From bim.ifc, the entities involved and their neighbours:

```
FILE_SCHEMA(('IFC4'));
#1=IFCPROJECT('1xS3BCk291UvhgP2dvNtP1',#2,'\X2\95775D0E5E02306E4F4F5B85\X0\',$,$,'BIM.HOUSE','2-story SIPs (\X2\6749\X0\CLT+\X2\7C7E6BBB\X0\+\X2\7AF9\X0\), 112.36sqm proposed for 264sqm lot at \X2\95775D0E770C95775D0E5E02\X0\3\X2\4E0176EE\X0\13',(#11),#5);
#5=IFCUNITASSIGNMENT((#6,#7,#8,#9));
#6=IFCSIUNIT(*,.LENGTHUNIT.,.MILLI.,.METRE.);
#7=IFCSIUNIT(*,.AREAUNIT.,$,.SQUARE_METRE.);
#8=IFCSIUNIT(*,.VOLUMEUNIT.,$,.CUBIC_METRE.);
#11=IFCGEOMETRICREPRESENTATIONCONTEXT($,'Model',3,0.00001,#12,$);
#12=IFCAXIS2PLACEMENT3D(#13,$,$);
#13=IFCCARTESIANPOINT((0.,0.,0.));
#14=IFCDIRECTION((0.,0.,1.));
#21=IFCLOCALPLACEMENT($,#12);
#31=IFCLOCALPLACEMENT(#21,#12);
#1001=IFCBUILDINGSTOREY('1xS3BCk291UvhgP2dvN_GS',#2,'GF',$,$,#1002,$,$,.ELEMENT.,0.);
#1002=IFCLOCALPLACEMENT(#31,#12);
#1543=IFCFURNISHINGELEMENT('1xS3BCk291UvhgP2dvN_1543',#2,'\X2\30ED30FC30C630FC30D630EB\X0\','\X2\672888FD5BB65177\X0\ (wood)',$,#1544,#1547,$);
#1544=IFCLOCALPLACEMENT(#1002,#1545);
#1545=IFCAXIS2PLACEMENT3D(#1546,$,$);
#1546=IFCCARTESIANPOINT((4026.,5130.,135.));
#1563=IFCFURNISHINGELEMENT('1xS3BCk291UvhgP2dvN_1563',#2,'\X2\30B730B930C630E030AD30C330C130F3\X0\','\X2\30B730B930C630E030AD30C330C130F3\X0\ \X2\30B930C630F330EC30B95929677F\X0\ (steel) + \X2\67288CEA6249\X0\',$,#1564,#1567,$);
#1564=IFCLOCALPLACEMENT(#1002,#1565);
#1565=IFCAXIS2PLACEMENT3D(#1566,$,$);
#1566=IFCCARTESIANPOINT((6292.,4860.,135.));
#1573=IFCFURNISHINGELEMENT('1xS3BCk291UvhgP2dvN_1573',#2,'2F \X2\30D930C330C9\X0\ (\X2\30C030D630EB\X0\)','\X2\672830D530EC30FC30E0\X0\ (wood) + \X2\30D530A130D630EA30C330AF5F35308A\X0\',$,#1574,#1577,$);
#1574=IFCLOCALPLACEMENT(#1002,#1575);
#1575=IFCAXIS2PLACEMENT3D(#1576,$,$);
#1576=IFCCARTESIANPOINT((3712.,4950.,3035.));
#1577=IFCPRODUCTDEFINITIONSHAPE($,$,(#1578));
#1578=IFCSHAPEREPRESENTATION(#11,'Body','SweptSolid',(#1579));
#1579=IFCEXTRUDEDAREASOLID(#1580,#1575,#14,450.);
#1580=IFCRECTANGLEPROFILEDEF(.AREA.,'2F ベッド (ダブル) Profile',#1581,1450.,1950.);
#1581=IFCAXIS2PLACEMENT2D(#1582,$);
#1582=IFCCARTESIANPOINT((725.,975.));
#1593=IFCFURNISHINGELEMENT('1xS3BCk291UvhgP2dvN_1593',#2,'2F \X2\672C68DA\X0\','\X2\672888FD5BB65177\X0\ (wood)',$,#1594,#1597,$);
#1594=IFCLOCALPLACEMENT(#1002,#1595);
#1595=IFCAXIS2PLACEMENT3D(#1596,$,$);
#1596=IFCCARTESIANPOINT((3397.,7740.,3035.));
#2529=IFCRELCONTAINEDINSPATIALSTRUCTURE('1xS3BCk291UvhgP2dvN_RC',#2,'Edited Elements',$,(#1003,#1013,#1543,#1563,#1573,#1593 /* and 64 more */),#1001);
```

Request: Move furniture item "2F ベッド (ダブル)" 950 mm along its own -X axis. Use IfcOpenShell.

```python
import ifcopenshell
import ifcopenshell.api.geometry
import ifcopenshell.util.placement
import ifcopenshell.util.unit

model = ifcopenshell.open("bim.ifc")
unit_scale = ifcopenshell.util.unit.calculate_unit_scale(model)

item = model.by_id(1573)
matrix = ifcopenshell.util.placement.get_local_placement(item.ObjectPlacement)
matrix[:3, 3] -= matrix[:3, 0] * 0.95 / unit_scale
ifcopenshell.api.geometry.edit_object_placement(model, product=item, matrix=matrix, is_si=False)

print(ifcopenshell.util.placement.get_local_placement(item.ObjectPlacement).round(3) + 0.0)

model.write("bim_edited.ifc")
```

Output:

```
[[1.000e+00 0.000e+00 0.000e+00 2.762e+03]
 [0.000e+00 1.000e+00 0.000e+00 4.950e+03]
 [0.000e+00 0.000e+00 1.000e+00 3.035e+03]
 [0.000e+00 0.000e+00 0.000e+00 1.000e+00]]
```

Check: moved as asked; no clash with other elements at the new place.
